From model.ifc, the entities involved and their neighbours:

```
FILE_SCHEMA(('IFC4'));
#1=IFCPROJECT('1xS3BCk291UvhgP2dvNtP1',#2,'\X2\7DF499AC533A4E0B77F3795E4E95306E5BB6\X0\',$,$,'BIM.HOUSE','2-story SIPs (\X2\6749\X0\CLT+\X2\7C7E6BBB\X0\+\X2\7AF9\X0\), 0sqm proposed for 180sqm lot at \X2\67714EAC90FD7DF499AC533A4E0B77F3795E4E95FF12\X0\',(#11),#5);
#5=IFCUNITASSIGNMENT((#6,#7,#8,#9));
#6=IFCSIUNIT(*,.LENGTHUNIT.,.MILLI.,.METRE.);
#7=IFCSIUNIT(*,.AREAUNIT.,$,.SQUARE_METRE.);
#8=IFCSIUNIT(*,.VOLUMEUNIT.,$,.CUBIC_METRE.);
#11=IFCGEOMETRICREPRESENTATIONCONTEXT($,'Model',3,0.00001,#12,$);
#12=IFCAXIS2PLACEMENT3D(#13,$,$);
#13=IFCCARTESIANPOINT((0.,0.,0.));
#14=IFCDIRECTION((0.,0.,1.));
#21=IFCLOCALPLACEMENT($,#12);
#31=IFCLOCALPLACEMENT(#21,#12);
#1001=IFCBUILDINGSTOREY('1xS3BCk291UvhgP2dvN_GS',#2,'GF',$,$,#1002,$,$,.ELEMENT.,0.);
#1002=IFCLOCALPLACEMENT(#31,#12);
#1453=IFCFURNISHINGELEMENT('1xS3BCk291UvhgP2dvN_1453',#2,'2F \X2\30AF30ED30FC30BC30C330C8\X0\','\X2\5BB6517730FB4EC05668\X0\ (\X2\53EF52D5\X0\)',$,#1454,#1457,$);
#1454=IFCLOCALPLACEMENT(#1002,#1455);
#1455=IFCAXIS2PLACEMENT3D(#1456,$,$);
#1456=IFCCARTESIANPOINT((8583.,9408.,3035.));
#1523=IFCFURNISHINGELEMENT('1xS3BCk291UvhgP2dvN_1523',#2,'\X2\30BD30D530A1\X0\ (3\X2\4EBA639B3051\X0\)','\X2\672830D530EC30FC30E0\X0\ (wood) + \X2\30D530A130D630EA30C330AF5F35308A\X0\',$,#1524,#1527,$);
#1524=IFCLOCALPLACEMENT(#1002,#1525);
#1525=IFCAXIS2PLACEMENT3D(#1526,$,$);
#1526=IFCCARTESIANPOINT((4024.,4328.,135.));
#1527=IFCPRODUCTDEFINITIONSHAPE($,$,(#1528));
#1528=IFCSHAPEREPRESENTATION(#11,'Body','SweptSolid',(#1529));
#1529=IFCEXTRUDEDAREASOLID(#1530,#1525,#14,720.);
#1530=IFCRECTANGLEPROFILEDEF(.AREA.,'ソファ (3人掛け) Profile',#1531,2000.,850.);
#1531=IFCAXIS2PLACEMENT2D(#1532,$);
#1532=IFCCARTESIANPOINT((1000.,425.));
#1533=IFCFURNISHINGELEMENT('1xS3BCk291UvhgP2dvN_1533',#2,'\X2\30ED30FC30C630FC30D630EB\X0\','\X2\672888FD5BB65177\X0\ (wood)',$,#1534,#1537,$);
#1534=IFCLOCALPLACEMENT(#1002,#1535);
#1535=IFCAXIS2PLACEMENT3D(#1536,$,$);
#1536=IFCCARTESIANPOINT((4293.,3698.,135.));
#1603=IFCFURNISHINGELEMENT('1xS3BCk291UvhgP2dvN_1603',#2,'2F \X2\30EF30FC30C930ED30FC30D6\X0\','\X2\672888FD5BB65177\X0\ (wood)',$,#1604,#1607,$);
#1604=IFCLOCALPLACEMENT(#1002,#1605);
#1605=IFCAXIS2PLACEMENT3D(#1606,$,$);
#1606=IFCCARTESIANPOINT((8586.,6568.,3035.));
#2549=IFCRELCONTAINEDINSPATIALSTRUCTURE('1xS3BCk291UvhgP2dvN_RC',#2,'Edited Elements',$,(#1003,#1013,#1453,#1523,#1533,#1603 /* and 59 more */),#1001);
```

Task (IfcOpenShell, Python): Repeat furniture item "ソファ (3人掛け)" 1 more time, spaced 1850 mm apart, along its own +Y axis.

```python
import ifcopenshell
import ifcopenshell.api.geometry
import ifcopenshell.api.root
import ifcopenshell.util.element
import ifcopenshell.util.placement

model = ifcopenshell.open("model.ifc")


def reuse_history(source, copy):
    """copy_class also copies each property set's owner history, people and application; keep the originals."""
    for rel in copy.IsDefinedBy:
        if rel.is_a("IfcRelDefinesByProperties") and (history := rel.RelatingPropertyDefinition.OwnerHistory):
            rel.RelatingPropertyDefinition.OwnerHistory = source.OwnerHistory
            ifcopenshell.util.element.remove_deep2(model, history)


source = model.by_guid("1xS3BCk291UvhgP2dvN_1523")
base = ifcopenshell.util.placement.get_local_placement(source.ObjectPlacement)
step = base[:3, 1] * 1850.0

for i in range(1, 2):
    copy = ifcopenshell.api.root.copy_class(model, product=source)
    copy.Representation = ifcopenshell.util.element.copy_deep(
        model, source.Representation, exclude=["IfcGeometricRepresentationContext", "IfcRepresentationMap"]
    )
    reuse_history(source, copy)
    matrix = base.copy()
    matrix[:3, 3] += i * step
    print("added at", matrix[:3, 3].round(3) + 0.0)
    ifcopenshell.api.geometry.edit_object_placement(model, product=copy, matrix=matrix, is_si=False)

model.write("model_updated.ifc")
```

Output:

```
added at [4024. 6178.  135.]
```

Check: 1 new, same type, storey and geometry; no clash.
